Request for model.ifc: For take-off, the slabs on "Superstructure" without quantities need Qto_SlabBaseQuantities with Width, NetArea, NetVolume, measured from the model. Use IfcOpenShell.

First a look at what the model holds.

```python
import ifcopenshell
import ifcopenshell.util.element
import ifcopenshell.util.unit

model = ifcopenshell.open("model.ifc")
print(model.schema)
for unit_type in ("LENGTHUNIT", "AREAUNIT", "VOLUMEUNIT"):
    print(unit_type, ifcopenshell.util.unit.calculate_unit_scale(model, unit_type))
storey = next(s for s in model.by_type("IfcBuildingStorey") if s.Name == "Superstructure")
slabs = [e for e in ifcopenshell.util.element.get_decomposition(storey) if e.is_a("IfcSlab")]
for e in sorted(slabs, key=lambda e: e.id()):
    print(e.id(), e.is_a(), e.Name, list(ifcopenshell.util.element.get_psets(e, qtos_only=True)), sep=" | ")
```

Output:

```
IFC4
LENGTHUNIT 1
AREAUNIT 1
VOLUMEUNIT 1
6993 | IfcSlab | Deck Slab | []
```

```python
import ifcopenshell
import ifcopenshell.api.pset
import ifcopenshell.geom
import ifcopenshell.util.element
import ifcopenshell.util.shape
import ifcopenshell.util.unit

model = ifcopenshell.open("model.ifc")
unit_scale = ifcopenshell.util.unit.calculate_unit_scale(model)
area_scale = ifcopenshell.util.unit.calculate_unit_scale(model, "AREAUNIT")
volume_scale = ifcopenshell.util.unit.calculate_unit_scale(model, "VOLUMEUNIT")
settings = ifcopenshell.geom.settings()

storey = next(s for s in model.by_type("IfcBuildingStorey") if s.Name == "Superstructure")
slabs = [e for e in ifcopenshell.util.element.get_decomposition(storey) if e.is_a("IfcSlab")]

for e in sorted(slabs, key=lambda e: e.id()):
    if ifcopenshell.util.element.get_psets(e, qtos_only=True, should_inherit=False):
        continue
    # Geometry comes back in metres, in the element's own axes.
    shape = ifcopenshell.geom.create_shape(settings, e)
    values = {
        "Width": ifcopenshell.util.shape.get_z(shape.geometry) / unit_scale,
        "NetArea": ifcopenshell.util.shape.get_footprint_area(shape.geometry) / area_scale,
        "NetVolume": ifcopenshell.util.shape.get_volume(shape.geometry) / volume_scale,
    }
    qto = ifcopenshell.api.pset.add_qto(model, product=e, name="Qto_SlabBaseQuantities")
    ifcopenshell.api.pset.edit_qto(model, qto=qto, properties=values)
    print(e.id(), {k: round(v, 3) for k, v in values.items()})

model.write("model_updated.ifc")
```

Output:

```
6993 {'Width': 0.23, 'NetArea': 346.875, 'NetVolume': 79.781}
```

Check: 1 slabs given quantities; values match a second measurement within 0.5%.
